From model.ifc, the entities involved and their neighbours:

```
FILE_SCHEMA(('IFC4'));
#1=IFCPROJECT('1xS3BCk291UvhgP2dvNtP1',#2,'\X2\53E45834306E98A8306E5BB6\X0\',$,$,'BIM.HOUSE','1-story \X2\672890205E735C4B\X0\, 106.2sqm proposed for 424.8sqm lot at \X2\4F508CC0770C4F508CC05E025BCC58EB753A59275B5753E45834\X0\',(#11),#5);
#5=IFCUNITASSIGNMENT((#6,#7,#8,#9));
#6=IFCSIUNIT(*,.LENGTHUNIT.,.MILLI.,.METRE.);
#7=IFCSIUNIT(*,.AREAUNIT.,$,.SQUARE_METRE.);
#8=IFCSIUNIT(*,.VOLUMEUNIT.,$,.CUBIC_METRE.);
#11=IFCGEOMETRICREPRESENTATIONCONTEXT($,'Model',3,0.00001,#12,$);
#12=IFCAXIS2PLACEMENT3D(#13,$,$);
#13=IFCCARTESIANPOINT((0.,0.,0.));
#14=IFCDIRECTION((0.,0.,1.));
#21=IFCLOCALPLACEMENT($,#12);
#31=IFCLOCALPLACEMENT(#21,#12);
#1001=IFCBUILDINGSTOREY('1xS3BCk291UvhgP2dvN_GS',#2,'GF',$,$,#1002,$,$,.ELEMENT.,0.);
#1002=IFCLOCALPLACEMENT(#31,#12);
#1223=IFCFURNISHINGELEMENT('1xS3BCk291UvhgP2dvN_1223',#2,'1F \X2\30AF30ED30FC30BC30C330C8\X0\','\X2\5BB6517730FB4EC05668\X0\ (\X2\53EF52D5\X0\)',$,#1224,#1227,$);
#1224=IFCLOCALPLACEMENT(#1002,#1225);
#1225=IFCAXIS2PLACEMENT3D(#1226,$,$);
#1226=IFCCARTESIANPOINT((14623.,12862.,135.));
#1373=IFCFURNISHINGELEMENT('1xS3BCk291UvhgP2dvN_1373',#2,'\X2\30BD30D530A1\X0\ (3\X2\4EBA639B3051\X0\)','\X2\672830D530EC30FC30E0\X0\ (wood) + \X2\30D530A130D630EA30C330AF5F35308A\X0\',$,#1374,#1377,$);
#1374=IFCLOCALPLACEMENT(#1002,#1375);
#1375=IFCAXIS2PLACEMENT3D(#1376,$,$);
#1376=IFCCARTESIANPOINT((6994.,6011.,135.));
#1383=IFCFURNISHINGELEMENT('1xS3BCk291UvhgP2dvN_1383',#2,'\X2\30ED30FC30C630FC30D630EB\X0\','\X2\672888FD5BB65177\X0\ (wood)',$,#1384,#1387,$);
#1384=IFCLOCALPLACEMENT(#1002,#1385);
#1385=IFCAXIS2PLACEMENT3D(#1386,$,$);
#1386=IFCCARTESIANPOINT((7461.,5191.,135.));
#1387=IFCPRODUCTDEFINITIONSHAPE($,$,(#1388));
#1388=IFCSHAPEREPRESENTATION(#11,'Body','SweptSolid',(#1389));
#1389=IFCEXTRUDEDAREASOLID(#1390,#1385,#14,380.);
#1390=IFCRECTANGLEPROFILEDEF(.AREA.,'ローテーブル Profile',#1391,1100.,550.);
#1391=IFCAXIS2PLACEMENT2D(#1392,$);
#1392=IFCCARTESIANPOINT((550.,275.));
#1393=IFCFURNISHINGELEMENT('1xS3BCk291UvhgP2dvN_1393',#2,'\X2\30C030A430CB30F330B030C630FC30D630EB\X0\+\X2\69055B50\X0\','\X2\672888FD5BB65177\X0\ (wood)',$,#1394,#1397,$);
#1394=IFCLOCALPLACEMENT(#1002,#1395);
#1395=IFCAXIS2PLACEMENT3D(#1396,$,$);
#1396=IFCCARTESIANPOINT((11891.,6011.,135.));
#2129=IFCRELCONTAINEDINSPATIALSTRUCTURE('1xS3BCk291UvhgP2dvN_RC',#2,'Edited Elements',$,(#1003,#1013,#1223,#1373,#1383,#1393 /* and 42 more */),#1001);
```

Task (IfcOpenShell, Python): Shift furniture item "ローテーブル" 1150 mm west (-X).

```python
import ifcopenshell
import ifcopenshell.api.geometry
import ifcopenshell.util.placement
import ifcopenshell.util.unit

model = ifcopenshell.open("model.ifc")
unit_scale = ifcopenshell.util.unit.calculate_unit_scale(model)

item = model.by_guid("1xS3BCk291UvhgP2dvN_1383")
matrix = ifcopenshell.util.placement.get_local_placement(item.ObjectPlacement)
matrix[0, 3] -= 1.15 / unit_scale
ifcopenshell.api.geometry.edit_object_placement(model, product=item, matrix=matrix, is_si=False)

print(ifcopenshell.util.placement.get_local_placement(item.ObjectPlacement).round(3) + 0.0)

model.write("model_edited.ifc")
```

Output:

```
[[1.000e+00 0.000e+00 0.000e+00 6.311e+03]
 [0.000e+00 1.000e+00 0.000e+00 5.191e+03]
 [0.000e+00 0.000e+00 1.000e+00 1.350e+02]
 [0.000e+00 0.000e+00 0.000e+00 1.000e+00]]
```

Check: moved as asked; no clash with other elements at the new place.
